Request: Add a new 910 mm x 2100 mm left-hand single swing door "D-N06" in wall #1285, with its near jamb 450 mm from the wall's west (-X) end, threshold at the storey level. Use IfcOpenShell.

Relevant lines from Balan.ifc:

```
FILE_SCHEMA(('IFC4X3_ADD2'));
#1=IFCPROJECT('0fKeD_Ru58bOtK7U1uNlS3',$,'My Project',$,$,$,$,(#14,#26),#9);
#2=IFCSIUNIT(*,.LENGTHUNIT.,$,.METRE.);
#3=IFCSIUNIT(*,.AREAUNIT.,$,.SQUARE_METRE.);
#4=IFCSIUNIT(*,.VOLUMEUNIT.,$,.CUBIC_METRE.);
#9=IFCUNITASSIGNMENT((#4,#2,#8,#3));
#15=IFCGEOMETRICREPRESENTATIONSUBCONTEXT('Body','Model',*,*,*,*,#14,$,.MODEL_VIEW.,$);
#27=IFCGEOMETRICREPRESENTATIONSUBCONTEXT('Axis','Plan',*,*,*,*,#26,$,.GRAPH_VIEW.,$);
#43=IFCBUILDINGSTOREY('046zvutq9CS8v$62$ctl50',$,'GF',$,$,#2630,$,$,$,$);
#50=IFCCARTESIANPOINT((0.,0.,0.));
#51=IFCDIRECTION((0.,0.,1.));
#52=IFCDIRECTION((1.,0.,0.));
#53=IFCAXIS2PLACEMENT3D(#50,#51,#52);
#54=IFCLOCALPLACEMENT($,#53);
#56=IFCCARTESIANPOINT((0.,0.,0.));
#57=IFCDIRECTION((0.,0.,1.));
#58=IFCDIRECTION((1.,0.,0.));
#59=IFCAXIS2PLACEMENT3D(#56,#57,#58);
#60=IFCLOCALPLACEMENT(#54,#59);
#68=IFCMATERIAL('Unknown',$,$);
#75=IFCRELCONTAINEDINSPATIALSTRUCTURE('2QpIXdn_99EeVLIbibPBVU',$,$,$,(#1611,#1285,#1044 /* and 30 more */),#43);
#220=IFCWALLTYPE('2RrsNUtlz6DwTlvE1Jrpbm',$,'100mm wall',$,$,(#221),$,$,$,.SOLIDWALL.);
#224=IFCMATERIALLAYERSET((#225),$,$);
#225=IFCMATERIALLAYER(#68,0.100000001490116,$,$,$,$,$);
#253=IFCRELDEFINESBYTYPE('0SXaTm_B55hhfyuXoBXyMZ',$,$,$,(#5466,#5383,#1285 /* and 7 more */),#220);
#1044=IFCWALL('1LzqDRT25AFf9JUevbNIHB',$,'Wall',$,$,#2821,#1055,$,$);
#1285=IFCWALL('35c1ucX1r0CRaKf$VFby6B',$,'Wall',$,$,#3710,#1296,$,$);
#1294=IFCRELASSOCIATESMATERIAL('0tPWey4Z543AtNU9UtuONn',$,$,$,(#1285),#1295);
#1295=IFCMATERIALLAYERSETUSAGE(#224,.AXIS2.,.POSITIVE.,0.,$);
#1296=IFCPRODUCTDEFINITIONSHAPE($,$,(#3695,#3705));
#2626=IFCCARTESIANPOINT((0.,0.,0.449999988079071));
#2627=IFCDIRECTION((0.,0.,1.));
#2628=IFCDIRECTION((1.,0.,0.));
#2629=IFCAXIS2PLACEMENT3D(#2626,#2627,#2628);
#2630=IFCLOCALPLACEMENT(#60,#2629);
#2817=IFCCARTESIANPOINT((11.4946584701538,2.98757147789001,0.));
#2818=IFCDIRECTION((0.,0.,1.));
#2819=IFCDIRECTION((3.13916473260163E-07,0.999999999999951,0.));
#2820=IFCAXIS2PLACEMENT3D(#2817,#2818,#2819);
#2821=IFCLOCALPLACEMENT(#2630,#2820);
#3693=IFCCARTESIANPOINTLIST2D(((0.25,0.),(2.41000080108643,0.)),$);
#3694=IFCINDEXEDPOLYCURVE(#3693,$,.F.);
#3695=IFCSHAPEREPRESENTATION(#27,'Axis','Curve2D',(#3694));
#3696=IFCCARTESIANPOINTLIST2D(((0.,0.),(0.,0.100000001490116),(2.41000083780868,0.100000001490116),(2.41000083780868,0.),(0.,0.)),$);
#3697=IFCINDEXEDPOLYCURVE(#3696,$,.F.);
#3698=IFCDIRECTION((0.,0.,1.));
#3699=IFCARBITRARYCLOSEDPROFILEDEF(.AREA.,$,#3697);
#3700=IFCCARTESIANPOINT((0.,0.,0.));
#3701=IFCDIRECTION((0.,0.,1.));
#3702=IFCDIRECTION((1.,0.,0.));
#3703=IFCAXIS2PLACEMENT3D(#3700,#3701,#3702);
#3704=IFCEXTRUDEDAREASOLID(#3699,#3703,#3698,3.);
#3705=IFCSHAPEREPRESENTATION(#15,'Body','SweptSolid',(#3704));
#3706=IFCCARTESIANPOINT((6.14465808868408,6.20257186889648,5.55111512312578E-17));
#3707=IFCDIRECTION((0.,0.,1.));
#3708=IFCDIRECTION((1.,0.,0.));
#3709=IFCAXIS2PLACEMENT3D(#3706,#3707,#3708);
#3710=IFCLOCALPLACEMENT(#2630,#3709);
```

```python
import numpy as np
import ifcopenshell
import ifcopenshell.api.feature
import ifcopenshell.api.geometry
import ifcopenshell.api.root
import ifcopenshell.api.spatial
import ifcopenshell.geom
import ifcopenshell.util.element
import ifcopenshell.util.placement
import ifcopenshell.util.representation
import ifcopenshell.util.shape
import ifcopenshell.util.unit

model = ifcopenshell.open("Balan.ifc")
unit_scale = ifcopenshell.util.unit.calculate_unit_scale(model)
settings = ifcopenshell.geom.settings()


def volume(element):
    """Net volume in cubic metres, openings subtracted."""
    shape = ifcopenshell.geom.create_shape(settings, element)
    return ifcopenshell.util.shape.get_volume(shape.geometry)


wall = model.by_guid("35c1ucX1r0CRaKf$VFby6B")
storey = ifcopenshell.util.element.get_container(wall, ifc_class="IfcBuildingStorey")
context = ifcopenshell.util.representation.get_context(model, "Model", "Body", "MODEL_VIEW")
before = volume(wall)

width, height, from_end, sill = 0.91, 2.1, 0.45, 0.0  # metres

# The wall runs along its own X axis, and the end named is its -X end.
wall_shape = ifcopenshell.geom.create_shape(settings, wall)
x, y, z = ifcopenshell.util.shape.get_vertices(wall_shape.geometry).T
start = x.min() + from_end
face, thickness = float(y.min()), float(y.max() - y.min())
wall_matrix = ifcopenshell.util.placement.get_local_placement(wall.ObjectPlacement)
level = ifcopenshell.util.placement.get_local_placement(storey.ObjectPlacement)[2, 3]


def in_wall(x, y):
    """Placement at x, y metres in the wall's axes, at sill height."""
    matrix = wall_matrix.copy()
    matrix[:, 3] = wall_matrix @ np.array([x / unit_scale, y / unit_scale, 0.0, 1.0])
    matrix[2, 3] = level + sill / unit_scale
    return matrix


# Opening: a box that overshoots both wall faces by 50 mm.
opening = ifcopenshell.api.root.create_entity(model, ifc_class="IfcOpeningElement", predefined_type="OPENING")
box = ifcopenshell.api.geometry.add_wall_representation(
    model, context=context, length=width, height=height, thickness=thickness + 0.1
)
ifcopenshell.api.geometry.assign_representation(model, product=opening, representation=box)
ifcopenshell.api.geometry.edit_object_placement(model, product=opening, matrix=in_wall(start, face - 0.05), is_si=False)
ifcopenshell.api.feature.add_feature(model, feature=opening, element=wall)

door = ifcopenshell.api.root.create_entity(model, ifc_class="IfcDoor", name="D-N06", predefined_type="DOOR")
door.OverallWidth, door.OverallHeight = width / unit_scale, height / unit_scale
door.OperationType = "SINGLE_SWING_LEFT"
body = ifcopenshell.api.geometry.add_door_representation(
    model,
    context=context,
    overall_width=door.OverallWidth,
    overall_height=door.OverallHeight,
    operation_type="SINGLE_SWING_LEFT",
    lining_properties={"LiningDepth": thickness / unit_scale, "ThresholdDepth": thickness / unit_scale},
)
ifcopenshell.api.geometry.assign_representation(model, product=door, representation=body)
ifcopenshell.api.spatial.assign_container(model, products=[door], relating_structure=storey)
ifcopenshell.api.feature.add_filling(model, opening=opening, element=door)

# The lining spans the wall, so the door starts at the wall face.
ifcopenshell.api.geometry.edit_object_placement(model, product=door, matrix=in_wall(start, face), is_si=False)

after = volume(wall)

print(f"wall volume {before:.3f} -> {after:.3f} m3")

model.write("Balan_v2.ifc")
```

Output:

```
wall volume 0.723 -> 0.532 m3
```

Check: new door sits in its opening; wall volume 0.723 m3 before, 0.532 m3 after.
